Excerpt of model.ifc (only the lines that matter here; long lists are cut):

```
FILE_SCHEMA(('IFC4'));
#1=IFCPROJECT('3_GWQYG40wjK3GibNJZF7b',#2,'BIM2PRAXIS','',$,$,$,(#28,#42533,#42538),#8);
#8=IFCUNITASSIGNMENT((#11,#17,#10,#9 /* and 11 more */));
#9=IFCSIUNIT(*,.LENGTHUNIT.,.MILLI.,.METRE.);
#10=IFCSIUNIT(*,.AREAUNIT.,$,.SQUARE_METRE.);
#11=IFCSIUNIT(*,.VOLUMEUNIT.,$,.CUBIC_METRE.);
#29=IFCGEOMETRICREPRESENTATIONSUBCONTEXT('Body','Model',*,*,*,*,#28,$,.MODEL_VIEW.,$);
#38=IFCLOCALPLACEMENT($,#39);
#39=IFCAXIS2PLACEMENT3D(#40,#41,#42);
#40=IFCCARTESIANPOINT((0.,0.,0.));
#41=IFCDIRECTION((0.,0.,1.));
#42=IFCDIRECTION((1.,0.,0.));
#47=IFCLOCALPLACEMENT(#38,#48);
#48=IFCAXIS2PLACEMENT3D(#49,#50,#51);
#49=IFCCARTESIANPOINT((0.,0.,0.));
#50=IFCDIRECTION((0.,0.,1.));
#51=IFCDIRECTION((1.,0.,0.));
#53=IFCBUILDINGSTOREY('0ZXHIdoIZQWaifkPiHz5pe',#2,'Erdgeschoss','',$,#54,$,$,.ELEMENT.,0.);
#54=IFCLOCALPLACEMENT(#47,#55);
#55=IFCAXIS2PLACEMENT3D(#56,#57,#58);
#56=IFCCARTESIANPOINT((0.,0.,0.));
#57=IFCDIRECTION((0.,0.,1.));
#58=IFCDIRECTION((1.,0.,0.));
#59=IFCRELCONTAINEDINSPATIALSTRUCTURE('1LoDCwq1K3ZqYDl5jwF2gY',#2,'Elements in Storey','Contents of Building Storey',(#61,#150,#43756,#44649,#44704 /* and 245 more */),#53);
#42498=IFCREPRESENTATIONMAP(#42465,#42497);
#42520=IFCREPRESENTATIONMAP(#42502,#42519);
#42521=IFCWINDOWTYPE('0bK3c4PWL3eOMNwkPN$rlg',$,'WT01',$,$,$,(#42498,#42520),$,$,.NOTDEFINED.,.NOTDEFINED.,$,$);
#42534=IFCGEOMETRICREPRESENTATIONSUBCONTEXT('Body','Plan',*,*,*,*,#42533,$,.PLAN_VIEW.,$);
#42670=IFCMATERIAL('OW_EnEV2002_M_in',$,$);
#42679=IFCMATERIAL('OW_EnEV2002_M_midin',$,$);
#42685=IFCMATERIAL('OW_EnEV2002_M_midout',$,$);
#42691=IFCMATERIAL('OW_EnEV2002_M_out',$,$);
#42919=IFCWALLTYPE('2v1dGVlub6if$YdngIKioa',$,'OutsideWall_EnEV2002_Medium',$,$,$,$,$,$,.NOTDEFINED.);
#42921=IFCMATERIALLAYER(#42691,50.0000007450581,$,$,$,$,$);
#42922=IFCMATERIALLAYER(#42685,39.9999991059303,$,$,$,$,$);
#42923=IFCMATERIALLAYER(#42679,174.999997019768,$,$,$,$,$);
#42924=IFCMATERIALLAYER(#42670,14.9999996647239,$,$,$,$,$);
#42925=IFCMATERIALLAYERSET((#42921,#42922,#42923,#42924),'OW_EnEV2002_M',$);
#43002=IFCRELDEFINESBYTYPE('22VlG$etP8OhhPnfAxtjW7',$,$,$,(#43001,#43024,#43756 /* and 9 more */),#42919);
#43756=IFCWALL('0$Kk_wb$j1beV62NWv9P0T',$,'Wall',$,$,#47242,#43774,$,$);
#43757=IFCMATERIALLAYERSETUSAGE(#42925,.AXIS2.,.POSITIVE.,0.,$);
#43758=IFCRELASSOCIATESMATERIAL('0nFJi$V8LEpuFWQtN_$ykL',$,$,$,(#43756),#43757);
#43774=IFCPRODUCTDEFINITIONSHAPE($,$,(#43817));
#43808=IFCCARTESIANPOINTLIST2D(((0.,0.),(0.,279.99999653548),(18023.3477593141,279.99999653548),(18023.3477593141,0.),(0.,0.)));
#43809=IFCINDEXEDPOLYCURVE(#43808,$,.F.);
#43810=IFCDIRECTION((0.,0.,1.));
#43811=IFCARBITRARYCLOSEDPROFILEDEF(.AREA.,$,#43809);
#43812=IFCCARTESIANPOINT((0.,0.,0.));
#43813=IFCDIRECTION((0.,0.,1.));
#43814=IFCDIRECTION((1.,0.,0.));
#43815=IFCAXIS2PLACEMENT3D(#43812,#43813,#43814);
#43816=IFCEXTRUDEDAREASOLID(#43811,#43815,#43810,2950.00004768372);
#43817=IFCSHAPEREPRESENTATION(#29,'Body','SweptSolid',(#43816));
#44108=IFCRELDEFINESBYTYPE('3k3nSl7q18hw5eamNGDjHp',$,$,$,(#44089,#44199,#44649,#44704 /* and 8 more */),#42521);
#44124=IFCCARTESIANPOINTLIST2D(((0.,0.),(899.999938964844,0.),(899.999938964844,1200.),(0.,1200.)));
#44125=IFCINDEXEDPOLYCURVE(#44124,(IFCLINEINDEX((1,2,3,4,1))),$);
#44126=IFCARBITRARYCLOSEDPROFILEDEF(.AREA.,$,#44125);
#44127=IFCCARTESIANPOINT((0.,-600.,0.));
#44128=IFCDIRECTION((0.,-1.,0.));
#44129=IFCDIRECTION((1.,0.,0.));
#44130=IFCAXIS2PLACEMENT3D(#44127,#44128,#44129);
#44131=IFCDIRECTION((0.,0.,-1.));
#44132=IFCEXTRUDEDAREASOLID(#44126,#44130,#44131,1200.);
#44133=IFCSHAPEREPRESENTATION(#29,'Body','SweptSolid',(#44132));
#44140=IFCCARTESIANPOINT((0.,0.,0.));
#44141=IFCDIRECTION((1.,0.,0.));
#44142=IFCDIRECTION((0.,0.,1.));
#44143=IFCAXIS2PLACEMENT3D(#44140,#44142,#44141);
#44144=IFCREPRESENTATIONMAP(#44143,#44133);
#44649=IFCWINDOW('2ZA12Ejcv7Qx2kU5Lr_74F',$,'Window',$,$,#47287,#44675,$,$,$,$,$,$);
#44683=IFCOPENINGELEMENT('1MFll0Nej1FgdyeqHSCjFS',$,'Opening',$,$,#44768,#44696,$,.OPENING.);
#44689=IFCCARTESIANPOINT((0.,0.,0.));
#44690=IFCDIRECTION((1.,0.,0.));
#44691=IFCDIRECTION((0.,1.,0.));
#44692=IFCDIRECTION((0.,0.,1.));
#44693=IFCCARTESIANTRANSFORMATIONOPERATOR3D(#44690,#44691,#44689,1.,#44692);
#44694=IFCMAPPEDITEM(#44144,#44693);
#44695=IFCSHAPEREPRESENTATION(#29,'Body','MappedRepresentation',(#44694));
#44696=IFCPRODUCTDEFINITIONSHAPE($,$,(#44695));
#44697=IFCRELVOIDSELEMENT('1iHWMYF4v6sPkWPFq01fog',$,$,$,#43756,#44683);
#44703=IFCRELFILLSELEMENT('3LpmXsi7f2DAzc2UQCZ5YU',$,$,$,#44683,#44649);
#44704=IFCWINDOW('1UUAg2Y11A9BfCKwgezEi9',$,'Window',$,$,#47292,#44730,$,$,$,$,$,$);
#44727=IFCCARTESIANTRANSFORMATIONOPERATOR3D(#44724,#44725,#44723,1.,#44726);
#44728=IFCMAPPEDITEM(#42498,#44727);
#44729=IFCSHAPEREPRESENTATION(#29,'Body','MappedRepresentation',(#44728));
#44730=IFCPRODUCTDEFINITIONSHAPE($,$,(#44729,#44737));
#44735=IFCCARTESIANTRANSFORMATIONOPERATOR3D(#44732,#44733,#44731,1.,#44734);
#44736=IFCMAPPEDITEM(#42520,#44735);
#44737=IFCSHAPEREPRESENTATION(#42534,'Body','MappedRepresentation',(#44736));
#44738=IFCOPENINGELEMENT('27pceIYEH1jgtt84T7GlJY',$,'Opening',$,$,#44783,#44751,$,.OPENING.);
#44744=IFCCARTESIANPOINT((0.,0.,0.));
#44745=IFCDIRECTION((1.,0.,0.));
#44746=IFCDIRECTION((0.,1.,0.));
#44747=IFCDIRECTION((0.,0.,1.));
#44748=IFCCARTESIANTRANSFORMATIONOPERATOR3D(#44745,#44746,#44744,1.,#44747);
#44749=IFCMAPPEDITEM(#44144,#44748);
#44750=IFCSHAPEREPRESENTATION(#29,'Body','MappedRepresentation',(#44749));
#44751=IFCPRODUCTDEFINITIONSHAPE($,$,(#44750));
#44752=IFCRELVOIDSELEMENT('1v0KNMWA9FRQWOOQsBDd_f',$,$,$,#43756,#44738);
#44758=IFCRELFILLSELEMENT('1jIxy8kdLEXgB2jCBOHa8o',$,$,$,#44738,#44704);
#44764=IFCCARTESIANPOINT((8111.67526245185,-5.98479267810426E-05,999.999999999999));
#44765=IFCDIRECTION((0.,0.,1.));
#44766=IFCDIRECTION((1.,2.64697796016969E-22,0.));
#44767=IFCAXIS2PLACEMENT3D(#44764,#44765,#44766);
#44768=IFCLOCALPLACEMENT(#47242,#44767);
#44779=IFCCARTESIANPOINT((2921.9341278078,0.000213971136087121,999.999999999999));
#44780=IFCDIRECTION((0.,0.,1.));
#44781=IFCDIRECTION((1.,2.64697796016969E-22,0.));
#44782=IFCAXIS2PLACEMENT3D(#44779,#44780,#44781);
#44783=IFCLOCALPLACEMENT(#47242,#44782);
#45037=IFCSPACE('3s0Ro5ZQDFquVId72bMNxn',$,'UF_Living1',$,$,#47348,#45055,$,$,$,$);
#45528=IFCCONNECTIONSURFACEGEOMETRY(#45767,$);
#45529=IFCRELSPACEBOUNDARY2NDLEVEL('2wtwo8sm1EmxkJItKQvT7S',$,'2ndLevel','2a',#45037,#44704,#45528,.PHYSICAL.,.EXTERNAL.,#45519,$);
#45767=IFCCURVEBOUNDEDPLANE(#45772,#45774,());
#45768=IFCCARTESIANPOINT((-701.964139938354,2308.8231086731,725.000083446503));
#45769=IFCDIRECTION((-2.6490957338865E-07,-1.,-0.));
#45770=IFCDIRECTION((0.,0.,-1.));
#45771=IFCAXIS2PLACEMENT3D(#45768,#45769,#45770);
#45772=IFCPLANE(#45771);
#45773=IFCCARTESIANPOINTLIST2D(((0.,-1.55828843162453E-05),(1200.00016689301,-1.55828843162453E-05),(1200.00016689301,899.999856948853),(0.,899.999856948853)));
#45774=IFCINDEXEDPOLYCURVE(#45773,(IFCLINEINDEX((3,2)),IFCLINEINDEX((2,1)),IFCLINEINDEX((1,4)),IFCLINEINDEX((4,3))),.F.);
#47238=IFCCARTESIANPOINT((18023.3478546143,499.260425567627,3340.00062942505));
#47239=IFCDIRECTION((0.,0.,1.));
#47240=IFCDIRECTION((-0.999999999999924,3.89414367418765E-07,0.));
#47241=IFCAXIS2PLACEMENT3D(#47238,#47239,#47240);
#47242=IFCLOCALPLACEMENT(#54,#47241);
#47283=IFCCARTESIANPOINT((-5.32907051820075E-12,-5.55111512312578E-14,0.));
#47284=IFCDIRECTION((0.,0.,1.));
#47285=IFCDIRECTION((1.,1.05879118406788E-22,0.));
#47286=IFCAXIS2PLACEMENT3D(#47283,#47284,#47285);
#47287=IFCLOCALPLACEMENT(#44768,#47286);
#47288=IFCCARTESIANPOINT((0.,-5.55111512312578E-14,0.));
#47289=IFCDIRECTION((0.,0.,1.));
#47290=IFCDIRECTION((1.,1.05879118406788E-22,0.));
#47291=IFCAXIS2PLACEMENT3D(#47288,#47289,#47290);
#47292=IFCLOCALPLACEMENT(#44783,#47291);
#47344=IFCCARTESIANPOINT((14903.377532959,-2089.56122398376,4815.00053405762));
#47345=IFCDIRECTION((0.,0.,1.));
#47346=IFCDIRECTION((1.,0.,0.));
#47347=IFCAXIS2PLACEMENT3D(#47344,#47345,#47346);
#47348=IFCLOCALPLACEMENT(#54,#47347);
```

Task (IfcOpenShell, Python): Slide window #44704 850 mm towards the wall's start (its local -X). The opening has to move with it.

```python
import numpy as np
import ifcopenshell
import ifcopenshell.api.geometry
import ifcopenshell.util.placement
import ifcopenshell.util.unit

model = ifcopenshell.open("model.ifc")
unit_scale = ifcopenshell.util.unit.calculate_unit_scale(model)

window = model.by_guid("1UUAg2Y11A9BfCKwgezEi9")
opening = window.FillsVoids[0].RelatingOpeningElement
wall = opening.VoidsElements[0].RelatingBuildingElement

wall_matrix = ifcopenshell.util.placement.get_local_placement(wall.ObjectPlacement)
shift = wall_matrix[:3, 0] * -0.85 / unit_scale
before = ifcopenshell.util.placement.get_local_placement(window.ObjectPlacement)[:3, 3].copy()

# The window is placed relative to its opening, so it follows when the opening moves.
matrix = ifcopenshell.util.placement.get_local_placement(opening.ObjectPlacement)
matrix[:3, 3] += shift
ifcopenshell.api.geometry.edit_object_placement(
    model, product=opening, matrix=matrix, is_si=False, should_transform_children=True
)

# Space boundary surfaces are stored in each space's coordinates; move them too.
for rel in window.ProvidesBoundaries:
    if not rel.ConnectionGeometry:
        continue
    surface = rel.ConnectionGeometry.SurfaceOnRelatingElement.BasisSurface
    space_matrix = ifcopenshell.util.placement.get_local_placement(rel.RelatingSpace.ObjectPlacement)
    point = np.array(surface.Position.Location.Coordinates) + space_matrix[:3, :3].T @ shift
    surface.Position = model.createIfcAxis2Placement3D(
        model.createIfcCartesianPoint(point.tolist()), surface.Position.Axis, surface.Position.RefDirection
    )

after = ifcopenshell.util.placement.get_local_placement(window.ObjectPlacement)[:3, 3]
print("window moved by", (after - before).round(3) + 0.0)

model.write("model_v2.ifc")
```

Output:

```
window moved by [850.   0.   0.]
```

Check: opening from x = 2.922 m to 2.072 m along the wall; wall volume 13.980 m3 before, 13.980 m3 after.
